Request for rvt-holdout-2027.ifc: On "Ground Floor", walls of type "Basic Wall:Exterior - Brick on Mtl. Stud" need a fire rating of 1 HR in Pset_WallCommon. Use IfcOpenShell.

First a look at what the model holds.

```python
import ifcopenshell
import ifcopenshell.util.element

model = ifcopenshell.open("rvt-holdout-2027.ifc")
print(model.schema)
storey = next(s for s in model.by_type("IfcBuildingStorey") if s.Name == "Ground Floor")
walls = [e for e in ifcopenshell.util.element.get_decomposition(storey) if e.is_a("IfcWall")]
seen = {}
for e in walls:
    element_type = ifcopenshell.util.element.get_type(e)
    key = (element_type.Name if element_type != e and element_type else None, ifcopenshell.util.element.get_pset(e, "Pset_WallCommon", "FireRating"))
    seen[key] = seen.get(key, 0) + 1
for (name, value), count in sorted(seen.items(), key=str):
    print(count, "x", name, "|", value)
```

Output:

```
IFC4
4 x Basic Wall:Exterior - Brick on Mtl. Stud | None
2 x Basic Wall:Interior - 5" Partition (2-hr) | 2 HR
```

```python
import ifcopenshell
import ifcopenshell.api.pset
import ifcopenshell.util.element

model = ifcopenshell.open("rvt-holdout-2027.ifc")

storey = next(s for s in model.by_type("IfcBuildingStorey") if s.Name == "Ground Floor")
walls = [e for e in ifcopenshell.util.element.get_decomposition(storey) if e.is_a("IfcWall")]

count = 0
for e in walls:
    element_type = ifcopenshell.util.element.get_type(e)
    if element_type in (None, e) or element_type.Name != "Basic Wall:Exterior - Brick on Mtl. Stud":
        continue
    # add_pset returns the element's existing set when there is one.
    pset = ifcopenshell.api.pset.add_pset(model, product=e, name="Pset_WallCommon")
    ifcopenshell.api.pset.edit_pset(model, pset=pset, properties={"FireRating": "1 HR"})
    count += 1

print(count, "walls updated")

model.write("rvt-holdout-2027_edited.ifc")
```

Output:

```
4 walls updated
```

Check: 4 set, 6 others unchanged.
